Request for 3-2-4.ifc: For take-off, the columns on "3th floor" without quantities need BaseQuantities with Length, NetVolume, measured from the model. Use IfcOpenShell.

First a look at what the model holds.

```python
import ifcopenshell
import ifcopenshell.util.element
import ifcopenshell.util.unit

model = ifcopenshell.open("3-2-4.ifc")
print(model.schema)
for unit_type in ("LENGTHUNIT", "AREAUNIT", "VOLUMEUNIT"):
    print(unit_type, ifcopenshell.util.unit.calculate_unit_scale(model, unit_type))
storey = next(s for s in model.by_type("IfcBuildingStorey") if s.Name == "3th floor")
columns = [e for e in ifcopenshell.util.element.get_decomposition(storey) if e.is_a("IfcColumn")]
for e in sorted(columns, key=lambda e: e.id()):
    print(e.id(), e.is_a(), e.Name, list(ifcopenshell.util.element.get_psets(e, qtos_only=True)), sep=" | ")
```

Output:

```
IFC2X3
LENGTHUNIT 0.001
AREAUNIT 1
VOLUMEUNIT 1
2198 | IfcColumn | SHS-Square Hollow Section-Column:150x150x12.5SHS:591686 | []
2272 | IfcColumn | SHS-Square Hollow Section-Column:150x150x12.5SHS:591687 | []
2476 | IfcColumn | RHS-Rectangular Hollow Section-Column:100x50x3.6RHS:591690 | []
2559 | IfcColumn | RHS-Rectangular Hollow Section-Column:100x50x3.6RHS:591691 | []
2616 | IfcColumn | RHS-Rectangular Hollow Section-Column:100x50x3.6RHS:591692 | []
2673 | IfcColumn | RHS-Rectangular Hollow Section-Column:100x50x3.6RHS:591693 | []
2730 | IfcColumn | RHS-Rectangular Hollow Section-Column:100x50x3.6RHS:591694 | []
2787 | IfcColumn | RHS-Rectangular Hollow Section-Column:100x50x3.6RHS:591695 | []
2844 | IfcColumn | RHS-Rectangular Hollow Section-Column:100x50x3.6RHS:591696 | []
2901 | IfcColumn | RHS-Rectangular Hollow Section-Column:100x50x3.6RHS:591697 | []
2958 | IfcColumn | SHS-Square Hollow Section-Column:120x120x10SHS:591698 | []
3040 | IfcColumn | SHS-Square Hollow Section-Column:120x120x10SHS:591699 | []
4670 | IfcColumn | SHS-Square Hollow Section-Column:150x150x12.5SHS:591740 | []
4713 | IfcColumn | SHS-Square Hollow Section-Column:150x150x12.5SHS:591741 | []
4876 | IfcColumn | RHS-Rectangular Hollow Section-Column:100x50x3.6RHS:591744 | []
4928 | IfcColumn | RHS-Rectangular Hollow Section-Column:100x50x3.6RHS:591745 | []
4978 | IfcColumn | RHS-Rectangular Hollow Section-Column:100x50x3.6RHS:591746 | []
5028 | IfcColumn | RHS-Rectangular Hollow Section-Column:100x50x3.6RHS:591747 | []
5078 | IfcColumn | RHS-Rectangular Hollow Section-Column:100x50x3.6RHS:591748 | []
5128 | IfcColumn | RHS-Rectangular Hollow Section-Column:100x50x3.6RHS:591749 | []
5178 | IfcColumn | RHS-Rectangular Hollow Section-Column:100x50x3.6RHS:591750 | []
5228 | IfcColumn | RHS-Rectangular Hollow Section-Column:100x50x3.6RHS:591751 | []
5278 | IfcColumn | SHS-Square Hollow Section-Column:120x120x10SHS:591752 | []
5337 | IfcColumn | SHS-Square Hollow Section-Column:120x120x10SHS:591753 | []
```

```python
import ifcopenshell
import ifcopenshell.api.pset
import ifcopenshell.geom
import ifcopenshell.util.element
import ifcopenshell.util.shape
import ifcopenshell.util.unit

model = ifcopenshell.open("3-2-4.ifc")
unit_scale = ifcopenshell.util.unit.calculate_unit_scale(model)
volume_scale = ifcopenshell.util.unit.calculate_unit_scale(model, "VOLUMEUNIT")
settings = ifcopenshell.geom.settings()

storey = next(s for s in model.by_type("IfcBuildingStorey") if s.Name == "3th floor")
columns = [e for e in ifcopenshell.util.element.get_decomposition(storey) if e.is_a("IfcColumn")]

for e in sorted(columns, key=lambda e: e.id()):
    if ifcopenshell.util.element.get_psets(e, qtos_only=True, should_inherit=False):
        continue
    # Geometry comes back in metres, in the element's own axes.
    shape = ifcopenshell.geom.create_shape(settings, e)
    values = {
        "Length": ifcopenshell.util.shape.get_z(shape.geometry) / unit_scale,
        "NetVolume": ifcopenshell.util.shape.get_volume(shape.geometry) / volume_scale,
    }
    qto = ifcopenshell.api.pset.add_qto(model, product=e, name="BaseQuantities")
    ifcopenshell.api.pset.edit_qto(model, qto=qto, properties=values)
    print(e.id(), {k: round(v, 3) for k, v in values.items()})

model.write("3-2-4_rev.ifc")
```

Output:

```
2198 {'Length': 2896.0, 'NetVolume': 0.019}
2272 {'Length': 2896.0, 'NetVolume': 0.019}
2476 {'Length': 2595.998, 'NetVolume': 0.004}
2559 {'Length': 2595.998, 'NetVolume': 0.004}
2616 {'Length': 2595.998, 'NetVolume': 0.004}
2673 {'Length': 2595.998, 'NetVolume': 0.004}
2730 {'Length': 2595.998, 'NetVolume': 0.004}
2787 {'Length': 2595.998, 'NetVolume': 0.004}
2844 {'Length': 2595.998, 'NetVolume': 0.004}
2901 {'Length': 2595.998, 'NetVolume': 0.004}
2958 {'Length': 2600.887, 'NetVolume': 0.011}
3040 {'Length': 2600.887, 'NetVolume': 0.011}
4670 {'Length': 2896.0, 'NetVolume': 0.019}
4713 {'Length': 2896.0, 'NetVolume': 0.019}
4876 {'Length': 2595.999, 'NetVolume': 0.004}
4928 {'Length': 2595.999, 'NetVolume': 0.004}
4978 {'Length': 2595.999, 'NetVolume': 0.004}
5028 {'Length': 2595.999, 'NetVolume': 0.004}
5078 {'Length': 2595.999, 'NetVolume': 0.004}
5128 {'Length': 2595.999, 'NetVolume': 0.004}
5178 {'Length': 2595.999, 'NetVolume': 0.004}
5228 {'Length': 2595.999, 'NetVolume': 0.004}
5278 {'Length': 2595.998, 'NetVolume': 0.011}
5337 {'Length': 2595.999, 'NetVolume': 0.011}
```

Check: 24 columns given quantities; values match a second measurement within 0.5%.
